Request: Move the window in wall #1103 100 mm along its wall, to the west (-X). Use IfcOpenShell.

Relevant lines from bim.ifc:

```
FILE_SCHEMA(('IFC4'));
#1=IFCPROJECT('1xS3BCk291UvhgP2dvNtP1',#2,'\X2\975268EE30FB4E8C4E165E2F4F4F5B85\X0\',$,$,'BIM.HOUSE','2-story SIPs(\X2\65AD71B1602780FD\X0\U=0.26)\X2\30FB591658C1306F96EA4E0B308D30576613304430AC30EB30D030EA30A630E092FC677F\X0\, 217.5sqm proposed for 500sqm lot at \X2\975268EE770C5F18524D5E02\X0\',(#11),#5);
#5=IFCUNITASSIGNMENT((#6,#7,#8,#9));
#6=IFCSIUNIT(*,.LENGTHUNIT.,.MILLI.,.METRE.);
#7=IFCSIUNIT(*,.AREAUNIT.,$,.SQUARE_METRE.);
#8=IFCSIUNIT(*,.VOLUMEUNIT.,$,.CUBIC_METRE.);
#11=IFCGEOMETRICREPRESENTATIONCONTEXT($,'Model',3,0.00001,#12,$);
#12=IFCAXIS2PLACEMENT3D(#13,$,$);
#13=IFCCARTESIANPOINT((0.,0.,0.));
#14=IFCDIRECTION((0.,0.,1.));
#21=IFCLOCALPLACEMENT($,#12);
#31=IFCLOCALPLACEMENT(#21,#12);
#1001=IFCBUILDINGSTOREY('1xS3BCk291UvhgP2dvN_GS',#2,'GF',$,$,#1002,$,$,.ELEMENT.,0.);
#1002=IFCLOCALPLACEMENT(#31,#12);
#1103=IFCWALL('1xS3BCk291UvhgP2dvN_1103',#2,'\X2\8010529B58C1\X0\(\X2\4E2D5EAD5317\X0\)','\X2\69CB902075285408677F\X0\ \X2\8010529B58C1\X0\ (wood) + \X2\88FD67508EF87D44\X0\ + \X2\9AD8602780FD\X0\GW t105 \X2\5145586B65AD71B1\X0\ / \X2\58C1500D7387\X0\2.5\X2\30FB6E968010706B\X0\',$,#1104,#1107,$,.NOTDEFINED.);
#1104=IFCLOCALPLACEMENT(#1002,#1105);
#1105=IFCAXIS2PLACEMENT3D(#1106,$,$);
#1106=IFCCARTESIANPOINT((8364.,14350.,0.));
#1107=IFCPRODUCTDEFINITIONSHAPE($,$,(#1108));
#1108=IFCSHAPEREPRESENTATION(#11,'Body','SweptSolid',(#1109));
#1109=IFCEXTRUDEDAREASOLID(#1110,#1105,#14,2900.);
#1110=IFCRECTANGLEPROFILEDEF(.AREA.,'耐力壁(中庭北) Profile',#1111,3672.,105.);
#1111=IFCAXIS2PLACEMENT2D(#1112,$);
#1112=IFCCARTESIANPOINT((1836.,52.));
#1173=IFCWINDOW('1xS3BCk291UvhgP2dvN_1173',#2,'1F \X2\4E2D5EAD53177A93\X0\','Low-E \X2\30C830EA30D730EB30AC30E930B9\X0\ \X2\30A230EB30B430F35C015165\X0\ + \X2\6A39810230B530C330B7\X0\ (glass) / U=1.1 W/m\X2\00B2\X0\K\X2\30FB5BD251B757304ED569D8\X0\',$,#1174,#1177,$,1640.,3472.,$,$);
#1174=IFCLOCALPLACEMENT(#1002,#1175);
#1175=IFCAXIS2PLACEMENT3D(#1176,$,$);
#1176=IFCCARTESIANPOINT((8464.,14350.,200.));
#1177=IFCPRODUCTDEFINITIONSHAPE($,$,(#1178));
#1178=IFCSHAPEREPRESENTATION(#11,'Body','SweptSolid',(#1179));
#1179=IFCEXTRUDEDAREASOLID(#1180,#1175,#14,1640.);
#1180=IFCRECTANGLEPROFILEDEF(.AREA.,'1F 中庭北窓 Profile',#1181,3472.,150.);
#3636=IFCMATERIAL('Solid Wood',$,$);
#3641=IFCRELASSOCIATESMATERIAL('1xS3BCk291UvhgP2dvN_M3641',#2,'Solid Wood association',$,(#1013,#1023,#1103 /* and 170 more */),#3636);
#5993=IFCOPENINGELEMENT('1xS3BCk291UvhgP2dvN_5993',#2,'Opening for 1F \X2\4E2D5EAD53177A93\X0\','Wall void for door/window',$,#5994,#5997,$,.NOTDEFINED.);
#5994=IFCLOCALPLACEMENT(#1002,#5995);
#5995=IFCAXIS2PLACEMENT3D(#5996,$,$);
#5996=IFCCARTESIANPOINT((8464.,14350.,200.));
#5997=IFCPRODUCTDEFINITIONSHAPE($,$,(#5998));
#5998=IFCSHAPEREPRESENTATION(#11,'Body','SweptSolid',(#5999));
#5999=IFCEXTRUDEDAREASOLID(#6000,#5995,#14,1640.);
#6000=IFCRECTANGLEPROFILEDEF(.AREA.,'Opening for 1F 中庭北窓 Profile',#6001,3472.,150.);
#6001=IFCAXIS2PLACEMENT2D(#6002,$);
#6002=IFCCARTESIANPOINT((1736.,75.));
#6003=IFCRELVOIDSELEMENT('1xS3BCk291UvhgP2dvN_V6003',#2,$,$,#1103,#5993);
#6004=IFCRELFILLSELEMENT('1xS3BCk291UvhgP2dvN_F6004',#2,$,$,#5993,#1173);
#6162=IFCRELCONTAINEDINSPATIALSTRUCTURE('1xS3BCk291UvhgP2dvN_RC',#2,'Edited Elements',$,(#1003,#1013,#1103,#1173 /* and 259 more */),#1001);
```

```python
import ifcopenshell
import ifcopenshell.api.geometry
import ifcopenshell.util.placement
import ifcopenshell.util.unit

model = ifcopenshell.open("bim.ifc")
unit_scale = ifcopenshell.util.unit.calculate_unit_scale(model)

window = model.by_guid("1xS3BCk291UvhgP2dvN_1173")
opening = window.FillsVoids[0].RelatingOpeningElement
wall = opening.VoidsElements[0].RelatingBuildingElement

wall_matrix = ifcopenshell.util.placement.get_local_placement(wall.ObjectPlacement)
shift = wall_matrix[:3, 0] * -0.1 / unit_scale
before = ifcopenshell.util.placement.get_local_placement(window.ObjectPlacement)[:3, 3].copy()

# The window is not placed relative to its opening, so move both.
for product in (opening, window):
    matrix = ifcopenshell.util.placement.get_local_placement(product.ObjectPlacement)
    matrix[:3, 3] += shift
    ifcopenshell.api.geometry.edit_object_placement(model, product=product, matrix=matrix, is_si=False)

after = ifcopenshell.util.placement.get_local_placement(window.ObjectPlacement)[:3, 3]
print("window moved by", (after - before).round(3) + 0.0)

model.write("bim_rev.ifc")
```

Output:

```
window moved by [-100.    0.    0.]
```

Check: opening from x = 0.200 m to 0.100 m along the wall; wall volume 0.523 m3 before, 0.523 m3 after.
